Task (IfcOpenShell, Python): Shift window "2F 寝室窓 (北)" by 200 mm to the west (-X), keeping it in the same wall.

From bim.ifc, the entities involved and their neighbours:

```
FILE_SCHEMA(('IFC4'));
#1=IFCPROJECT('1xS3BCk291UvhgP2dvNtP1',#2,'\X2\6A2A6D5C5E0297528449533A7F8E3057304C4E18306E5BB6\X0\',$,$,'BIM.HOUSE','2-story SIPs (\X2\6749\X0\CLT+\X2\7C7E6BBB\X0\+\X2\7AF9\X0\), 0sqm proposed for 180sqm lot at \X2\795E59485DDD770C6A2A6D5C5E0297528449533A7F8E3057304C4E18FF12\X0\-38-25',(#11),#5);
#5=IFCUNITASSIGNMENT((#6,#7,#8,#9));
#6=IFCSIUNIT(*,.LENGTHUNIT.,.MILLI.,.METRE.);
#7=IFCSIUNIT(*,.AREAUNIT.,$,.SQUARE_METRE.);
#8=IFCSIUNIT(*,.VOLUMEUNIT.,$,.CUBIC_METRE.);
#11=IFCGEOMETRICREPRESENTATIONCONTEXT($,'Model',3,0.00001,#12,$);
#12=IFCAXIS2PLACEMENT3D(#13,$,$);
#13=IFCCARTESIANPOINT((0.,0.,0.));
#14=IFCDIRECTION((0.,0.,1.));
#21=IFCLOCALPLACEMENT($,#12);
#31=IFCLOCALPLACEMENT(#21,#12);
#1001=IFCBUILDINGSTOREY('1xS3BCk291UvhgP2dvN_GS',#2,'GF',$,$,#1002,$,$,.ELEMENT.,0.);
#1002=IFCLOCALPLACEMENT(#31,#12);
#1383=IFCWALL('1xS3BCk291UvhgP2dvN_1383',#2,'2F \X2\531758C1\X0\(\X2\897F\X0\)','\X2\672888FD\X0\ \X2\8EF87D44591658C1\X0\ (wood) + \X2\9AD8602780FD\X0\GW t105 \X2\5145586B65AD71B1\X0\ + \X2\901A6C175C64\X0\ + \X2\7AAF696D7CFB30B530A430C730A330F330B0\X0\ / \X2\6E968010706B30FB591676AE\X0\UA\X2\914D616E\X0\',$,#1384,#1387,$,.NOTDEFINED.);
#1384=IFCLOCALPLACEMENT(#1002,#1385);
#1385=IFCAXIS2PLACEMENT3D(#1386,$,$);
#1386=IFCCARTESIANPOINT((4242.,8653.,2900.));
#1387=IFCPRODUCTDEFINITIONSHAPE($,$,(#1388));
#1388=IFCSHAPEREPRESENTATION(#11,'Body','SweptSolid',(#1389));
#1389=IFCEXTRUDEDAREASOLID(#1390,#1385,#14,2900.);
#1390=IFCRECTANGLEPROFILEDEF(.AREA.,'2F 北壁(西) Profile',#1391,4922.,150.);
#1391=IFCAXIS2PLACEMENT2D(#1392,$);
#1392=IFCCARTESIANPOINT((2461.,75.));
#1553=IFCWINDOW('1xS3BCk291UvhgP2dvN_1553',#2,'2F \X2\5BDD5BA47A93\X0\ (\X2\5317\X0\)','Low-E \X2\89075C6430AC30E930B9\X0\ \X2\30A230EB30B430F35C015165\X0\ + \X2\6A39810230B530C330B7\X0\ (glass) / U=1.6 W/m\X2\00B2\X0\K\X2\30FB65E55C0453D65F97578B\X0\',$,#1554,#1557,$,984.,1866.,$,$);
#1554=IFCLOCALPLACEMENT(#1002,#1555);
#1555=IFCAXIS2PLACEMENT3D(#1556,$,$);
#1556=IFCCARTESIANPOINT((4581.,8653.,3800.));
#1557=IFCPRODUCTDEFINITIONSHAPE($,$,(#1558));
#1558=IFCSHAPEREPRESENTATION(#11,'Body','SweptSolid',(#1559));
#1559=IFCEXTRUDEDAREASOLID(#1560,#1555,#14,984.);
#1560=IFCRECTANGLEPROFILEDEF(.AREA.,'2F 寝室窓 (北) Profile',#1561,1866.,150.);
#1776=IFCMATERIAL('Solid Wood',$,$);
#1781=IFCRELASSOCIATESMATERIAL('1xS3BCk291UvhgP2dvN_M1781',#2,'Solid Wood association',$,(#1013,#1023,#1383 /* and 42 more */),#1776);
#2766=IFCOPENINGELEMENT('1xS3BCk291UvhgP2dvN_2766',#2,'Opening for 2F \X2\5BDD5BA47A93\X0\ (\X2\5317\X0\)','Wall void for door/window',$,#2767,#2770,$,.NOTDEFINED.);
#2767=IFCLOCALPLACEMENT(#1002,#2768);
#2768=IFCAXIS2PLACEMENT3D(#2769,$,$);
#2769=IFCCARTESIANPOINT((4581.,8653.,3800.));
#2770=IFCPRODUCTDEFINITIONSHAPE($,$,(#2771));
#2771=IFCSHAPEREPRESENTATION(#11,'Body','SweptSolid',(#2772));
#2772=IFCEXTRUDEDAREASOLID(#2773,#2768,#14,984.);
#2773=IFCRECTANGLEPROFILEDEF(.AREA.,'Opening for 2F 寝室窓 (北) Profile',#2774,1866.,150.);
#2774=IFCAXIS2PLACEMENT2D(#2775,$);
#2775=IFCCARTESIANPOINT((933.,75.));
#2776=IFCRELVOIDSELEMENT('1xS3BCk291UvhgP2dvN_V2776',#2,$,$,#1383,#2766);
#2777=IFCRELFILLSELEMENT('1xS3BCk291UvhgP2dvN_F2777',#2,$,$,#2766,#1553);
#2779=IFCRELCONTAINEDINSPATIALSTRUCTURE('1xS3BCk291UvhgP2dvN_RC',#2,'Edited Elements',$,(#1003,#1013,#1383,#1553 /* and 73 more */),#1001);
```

```python
import ifcopenshell
import ifcopenshell.api.geometry
import ifcopenshell.util.placement
import ifcopenshell.util.unit

model = ifcopenshell.open("bim.ifc")
unit_scale = ifcopenshell.util.unit.calculate_unit_scale(model)

window = model.by_guid("1xS3BCk291UvhgP2dvN_1553")
opening = window.FillsVoids[0].RelatingOpeningElement
wall = opening.VoidsElements[0].RelatingBuildingElement

wall_matrix = ifcopenshell.util.placement.get_local_placement(wall.ObjectPlacement)
shift = wall_matrix[:3, 0] * -0.2 / unit_scale
before = ifcopenshell.util.placement.get_local_placement(window.ObjectPlacement)[:3, 3].copy()

# The window is not placed relative to its opening, so move both.
for product in (opening, window):
    matrix = ifcopenshell.util.placement.get_local_placement(product.ObjectPlacement)
    matrix[:3, 3] += shift
    ifcopenshell.api.geometry.edit_object_placement(model, product=product, matrix=matrix, is_si=False)

after = ifcopenshell.util.placement.get_local_placement(window.ObjectPlacement)[:3, 3]
print("window moved by", (after - before).round(3) + 0.0)

model.write("bim_rev.ifc")
```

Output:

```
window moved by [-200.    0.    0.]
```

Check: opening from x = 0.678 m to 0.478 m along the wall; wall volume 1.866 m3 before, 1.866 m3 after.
